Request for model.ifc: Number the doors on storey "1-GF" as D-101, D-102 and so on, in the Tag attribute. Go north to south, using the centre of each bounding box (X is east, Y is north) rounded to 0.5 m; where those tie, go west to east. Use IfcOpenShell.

First a look at what the model holds.

```python
import ifcopenshell
import ifcopenshell.util.element
import ifcopenshell.util.placement

model = ifcopenshell.open("model.ifc")
print(model.schema)
storey = next(s for s in model.by_type("IfcBuildingStorey") if s.Name == "1-GF")
doors = [e for e in ifcopenshell.util.element.get_decomposition(storey) if e.is_a("IfcDoor")]
for e in sorted(doors, key=lambda e: e.id()):
    origin = ifcopenshell.util.placement.get_local_placement(e.ObjectPlacement)[:3, 3]
    print(e.id(), e.Tag, e.Name, origin.round(2) + 0.0, sep=" | ")
```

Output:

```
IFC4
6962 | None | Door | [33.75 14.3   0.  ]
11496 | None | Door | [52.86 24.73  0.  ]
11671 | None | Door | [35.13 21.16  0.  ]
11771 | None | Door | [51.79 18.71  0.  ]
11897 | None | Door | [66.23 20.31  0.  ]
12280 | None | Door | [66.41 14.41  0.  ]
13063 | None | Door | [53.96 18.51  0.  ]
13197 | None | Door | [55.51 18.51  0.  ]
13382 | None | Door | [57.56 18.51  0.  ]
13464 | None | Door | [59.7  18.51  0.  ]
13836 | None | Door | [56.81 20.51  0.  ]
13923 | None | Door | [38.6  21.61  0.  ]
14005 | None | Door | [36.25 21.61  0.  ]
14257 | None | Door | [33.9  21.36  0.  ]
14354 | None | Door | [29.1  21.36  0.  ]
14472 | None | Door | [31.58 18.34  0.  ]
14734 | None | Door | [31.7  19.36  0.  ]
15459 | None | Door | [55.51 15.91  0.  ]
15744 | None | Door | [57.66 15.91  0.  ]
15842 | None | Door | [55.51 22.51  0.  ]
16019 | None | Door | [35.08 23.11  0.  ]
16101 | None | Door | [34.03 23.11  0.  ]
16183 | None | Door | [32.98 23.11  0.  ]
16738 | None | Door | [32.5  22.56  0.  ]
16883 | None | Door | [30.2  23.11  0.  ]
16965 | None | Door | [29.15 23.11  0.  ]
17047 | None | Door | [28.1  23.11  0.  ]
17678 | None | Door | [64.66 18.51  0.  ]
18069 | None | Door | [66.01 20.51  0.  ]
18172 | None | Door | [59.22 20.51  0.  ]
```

```python
import ifcopenshell
import ifcopenshell.geom
import ifcopenshell.util.element
import ifcopenshell.util.shape

model = ifcopenshell.open("model.ifc")
settings = ifcopenshell.geom.settings()
settings.set("use-world-coords", True)


def centre(element):
    shape = ifcopenshell.geom.create_shape(settings, element)
    return ifcopenshell.util.shape.get_bbox_centroid(shape.geometry)


storey = next(s for s in model.by_type("IfcBuildingStorey") if s.Name == "1-GF")
doors = [e for e in ifcopenshell.util.element.get_decomposition(storey) if e.is_a("IfcDoor")]

# Insertion points can sit at a corner or the storey origin, so sort by the geometry (in metres).
centres = {e: centre(e) for e in doors}
doors.sort(key=lambda e: (-round(centres[e][1] / 0.5), centres[e][0]))

for i, e in enumerate(doors, start=1):
    number = f"D-1{i:02d}"
    e.Tag = number
    print(e.id(), number)

model.write("model_updated.ifc")
```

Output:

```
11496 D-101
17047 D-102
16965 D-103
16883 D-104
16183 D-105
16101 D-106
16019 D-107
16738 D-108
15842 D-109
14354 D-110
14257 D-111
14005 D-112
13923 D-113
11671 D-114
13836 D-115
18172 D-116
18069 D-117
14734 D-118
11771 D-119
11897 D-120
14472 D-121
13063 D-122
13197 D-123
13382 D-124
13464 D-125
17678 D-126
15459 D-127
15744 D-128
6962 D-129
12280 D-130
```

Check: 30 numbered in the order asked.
